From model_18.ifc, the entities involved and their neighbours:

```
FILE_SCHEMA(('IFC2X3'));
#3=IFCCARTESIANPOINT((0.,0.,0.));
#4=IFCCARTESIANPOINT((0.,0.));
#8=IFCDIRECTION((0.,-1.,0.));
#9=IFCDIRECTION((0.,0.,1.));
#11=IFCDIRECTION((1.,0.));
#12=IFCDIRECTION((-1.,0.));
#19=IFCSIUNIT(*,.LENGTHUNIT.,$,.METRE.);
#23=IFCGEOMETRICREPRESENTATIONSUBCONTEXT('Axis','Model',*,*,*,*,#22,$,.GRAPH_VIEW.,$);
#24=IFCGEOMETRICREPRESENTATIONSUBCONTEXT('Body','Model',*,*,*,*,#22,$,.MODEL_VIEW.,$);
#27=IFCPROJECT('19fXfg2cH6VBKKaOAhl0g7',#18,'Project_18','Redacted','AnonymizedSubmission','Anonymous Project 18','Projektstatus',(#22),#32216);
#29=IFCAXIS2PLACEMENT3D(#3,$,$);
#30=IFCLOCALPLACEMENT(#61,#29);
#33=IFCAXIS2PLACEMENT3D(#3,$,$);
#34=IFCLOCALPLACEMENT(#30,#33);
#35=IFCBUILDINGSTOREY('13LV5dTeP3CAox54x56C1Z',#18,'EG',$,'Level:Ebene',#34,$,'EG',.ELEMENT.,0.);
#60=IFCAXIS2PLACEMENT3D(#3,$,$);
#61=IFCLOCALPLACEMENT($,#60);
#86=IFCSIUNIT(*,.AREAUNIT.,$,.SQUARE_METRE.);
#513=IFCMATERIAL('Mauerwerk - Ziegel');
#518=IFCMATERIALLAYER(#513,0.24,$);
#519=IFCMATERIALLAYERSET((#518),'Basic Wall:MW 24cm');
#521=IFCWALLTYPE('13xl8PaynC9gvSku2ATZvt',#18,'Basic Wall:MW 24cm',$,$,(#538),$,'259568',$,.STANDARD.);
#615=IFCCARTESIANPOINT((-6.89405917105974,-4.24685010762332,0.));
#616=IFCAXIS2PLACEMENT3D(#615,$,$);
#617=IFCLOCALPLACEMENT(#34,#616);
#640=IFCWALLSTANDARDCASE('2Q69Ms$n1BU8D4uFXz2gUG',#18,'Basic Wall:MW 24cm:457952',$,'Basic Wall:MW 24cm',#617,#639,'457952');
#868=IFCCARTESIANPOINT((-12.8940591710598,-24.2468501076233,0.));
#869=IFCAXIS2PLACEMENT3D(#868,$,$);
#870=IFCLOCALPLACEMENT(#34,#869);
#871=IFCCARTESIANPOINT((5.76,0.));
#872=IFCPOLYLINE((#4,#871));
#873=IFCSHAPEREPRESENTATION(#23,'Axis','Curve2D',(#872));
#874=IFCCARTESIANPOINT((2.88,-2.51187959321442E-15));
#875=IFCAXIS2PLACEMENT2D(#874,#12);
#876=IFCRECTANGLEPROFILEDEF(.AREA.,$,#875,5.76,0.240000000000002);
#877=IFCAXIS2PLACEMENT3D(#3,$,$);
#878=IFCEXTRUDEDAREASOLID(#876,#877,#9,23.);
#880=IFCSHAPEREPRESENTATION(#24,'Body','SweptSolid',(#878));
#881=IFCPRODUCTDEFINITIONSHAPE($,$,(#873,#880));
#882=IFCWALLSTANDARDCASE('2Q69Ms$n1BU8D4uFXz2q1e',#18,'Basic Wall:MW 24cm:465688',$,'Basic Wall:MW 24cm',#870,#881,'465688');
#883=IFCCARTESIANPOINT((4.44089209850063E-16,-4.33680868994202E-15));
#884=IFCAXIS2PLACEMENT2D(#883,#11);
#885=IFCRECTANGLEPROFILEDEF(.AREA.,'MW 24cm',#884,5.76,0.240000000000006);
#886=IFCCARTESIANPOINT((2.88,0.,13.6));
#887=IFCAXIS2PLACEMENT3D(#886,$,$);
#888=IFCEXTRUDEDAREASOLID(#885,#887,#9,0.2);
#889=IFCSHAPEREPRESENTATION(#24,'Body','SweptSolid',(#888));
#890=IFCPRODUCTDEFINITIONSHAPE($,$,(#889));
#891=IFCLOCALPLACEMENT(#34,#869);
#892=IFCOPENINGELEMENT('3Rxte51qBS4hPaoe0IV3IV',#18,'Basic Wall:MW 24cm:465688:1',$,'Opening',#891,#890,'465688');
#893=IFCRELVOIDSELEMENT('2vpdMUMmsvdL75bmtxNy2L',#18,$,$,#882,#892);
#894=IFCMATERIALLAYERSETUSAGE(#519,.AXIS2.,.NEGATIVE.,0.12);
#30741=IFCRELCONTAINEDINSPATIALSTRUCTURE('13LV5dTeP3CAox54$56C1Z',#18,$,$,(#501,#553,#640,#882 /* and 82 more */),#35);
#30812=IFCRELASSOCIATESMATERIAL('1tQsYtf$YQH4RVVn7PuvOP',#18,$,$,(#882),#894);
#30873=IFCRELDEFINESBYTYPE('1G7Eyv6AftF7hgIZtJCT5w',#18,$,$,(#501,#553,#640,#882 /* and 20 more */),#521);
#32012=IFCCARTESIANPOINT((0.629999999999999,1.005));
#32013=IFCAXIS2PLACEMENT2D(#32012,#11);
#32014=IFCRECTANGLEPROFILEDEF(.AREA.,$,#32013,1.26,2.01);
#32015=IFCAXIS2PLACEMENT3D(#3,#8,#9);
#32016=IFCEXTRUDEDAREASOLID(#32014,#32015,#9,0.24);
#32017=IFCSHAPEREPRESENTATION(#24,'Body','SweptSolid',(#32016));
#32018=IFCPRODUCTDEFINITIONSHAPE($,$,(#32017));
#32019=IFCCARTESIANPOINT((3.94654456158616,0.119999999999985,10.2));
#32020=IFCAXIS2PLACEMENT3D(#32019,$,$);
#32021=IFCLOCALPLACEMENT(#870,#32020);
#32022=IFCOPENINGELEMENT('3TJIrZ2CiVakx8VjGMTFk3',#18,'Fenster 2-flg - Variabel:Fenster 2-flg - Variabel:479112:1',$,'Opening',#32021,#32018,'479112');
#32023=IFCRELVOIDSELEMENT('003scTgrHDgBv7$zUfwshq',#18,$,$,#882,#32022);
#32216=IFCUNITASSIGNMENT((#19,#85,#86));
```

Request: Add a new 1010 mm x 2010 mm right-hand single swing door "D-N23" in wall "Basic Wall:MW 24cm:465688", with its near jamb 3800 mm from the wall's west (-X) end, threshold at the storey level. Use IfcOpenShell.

```python
import numpy as np
import ifcopenshell
import ifcopenshell.api.feature
import ifcopenshell.api.geometry
import ifcopenshell.api.root
import ifcopenshell.api.spatial
import ifcopenshell.api.type
import ifcopenshell.geom
import ifcopenshell.util.element
import ifcopenshell.util.placement
import ifcopenshell.util.representation
import ifcopenshell.util.shape
import ifcopenshell.util.unit

model = ifcopenshell.open("model_18.ifc")
unit_scale = ifcopenshell.util.unit.calculate_unit_scale(model)
settings = ifcopenshell.geom.settings()


def volume(element):
    """Net volume in cubic metres, openings subtracted."""
    shape = ifcopenshell.geom.create_shape(settings, element)
    return ifcopenshell.util.shape.get_volume(shape.geometry)


wall = model.by_guid("2Q69Ms$n1BU8D4uFXz2q1e")
storey = ifcopenshell.util.element.get_container(wall, ifc_class="IfcBuildingStorey")
context = ifcopenshell.util.representation.get_context(model, "Model", "Body", "MODEL_VIEW")
before = volume(wall)

width, height, from_end, sill = 1.01, 2.01, 3.8, 0.0  # metres

# The wall runs along its own X axis, and the end named is its -X end.
wall_shape = ifcopenshell.geom.create_shape(settings, wall)
x, y, z = ifcopenshell.util.shape.get_vertices(wall_shape.geometry).T
start = x.min() + from_end
face, thickness = float(y.min()), float(y.max() - y.min())
wall_matrix = ifcopenshell.util.placement.get_local_placement(wall.ObjectPlacement)
level = ifcopenshell.util.placement.get_local_placement(storey.ObjectPlacement)[2, 3]


def in_wall(x, y):
    """Placement at x, y metres in the wall's axes, at sill height."""
    matrix = wall_matrix.copy()
    matrix[:, 3] = wall_matrix @ np.array([x / unit_scale, y / unit_scale, 0.0, 1.0])
    matrix[2, 3] = level + sill / unit_scale
    return matrix


# Opening: a box that overshoots both wall faces by 50 mm.
opening = ifcopenshell.api.root.create_entity(model, ifc_class="IfcOpeningElement")
box = ifcopenshell.api.geometry.add_wall_representation(
    model, context=context, length=width, height=height, thickness=thickness + 0.1
)
ifcopenshell.api.geometry.assign_representation(model, product=opening, representation=box)
ifcopenshell.api.geometry.edit_object_placement(model, product=opening, matrix=in_wall(start, face - 0.05), is_si=False)
ifcopenshell.api.feature.add_feature(model, feature=opening, element=wall)

door = ifcopenshell.api.root.create_entity(model, ifc_class="IfcDoor", name="D-N23")
door.OverallWidth, door.OverallHeight = width / unit_scale, height / unit_scale
body = ifcopenshell.api.geometry.add_door_representation(
    model,
    context=context,
    overall_width=door.OverallWidth,
    overall_height=door.OverallHeight,
    operation_type="SINGLE_SWING_RIGHT",
    lining_properties={"LiningDepth": thickness / unit_scale, "ThresholdDepth": thickness / unit_scale},
)
ifcopenshell.api.geometry.assign_representation(model, product=door, representation=body)
ifcopenshell.api.spatial.assign_container(model, products=[door], relating_structure=storey)
fills = ifcopenshell.api.feature.add_filling(model, opening=opening, element=door)
fills.OwnerHistory = door.OwnerHistory  # required in IFC2X3

# IFC2X3 keeps the operation on the door style.
style = ifcopenshell.api.root.create_entity(model, ifc_class="IfcDoorStyle", name="D-N23")
style.OperationType, style.ConstructionType = "SINGLE_SWING_RIGHT", "NOTDEFINED"
style.ParameterTakesPrecedence = style.Sizeable = False
ifcopenshell.api.type.assign_type(model, related_objects=[door], relating_type=style)

# The lining spans the wall, so the door starts at the wall face.
ifcopenshell.api.geometry.edit_object_placement(model, product=door, matrix=in_wall(start, face), is_si=False)

after = volume(wall)

print(f"wall volume {before:.3f} -> {after:.3f} m3")

model.write("model_18_v2.ifc")
```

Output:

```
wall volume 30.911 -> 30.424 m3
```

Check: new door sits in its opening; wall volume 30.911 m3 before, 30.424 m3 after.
